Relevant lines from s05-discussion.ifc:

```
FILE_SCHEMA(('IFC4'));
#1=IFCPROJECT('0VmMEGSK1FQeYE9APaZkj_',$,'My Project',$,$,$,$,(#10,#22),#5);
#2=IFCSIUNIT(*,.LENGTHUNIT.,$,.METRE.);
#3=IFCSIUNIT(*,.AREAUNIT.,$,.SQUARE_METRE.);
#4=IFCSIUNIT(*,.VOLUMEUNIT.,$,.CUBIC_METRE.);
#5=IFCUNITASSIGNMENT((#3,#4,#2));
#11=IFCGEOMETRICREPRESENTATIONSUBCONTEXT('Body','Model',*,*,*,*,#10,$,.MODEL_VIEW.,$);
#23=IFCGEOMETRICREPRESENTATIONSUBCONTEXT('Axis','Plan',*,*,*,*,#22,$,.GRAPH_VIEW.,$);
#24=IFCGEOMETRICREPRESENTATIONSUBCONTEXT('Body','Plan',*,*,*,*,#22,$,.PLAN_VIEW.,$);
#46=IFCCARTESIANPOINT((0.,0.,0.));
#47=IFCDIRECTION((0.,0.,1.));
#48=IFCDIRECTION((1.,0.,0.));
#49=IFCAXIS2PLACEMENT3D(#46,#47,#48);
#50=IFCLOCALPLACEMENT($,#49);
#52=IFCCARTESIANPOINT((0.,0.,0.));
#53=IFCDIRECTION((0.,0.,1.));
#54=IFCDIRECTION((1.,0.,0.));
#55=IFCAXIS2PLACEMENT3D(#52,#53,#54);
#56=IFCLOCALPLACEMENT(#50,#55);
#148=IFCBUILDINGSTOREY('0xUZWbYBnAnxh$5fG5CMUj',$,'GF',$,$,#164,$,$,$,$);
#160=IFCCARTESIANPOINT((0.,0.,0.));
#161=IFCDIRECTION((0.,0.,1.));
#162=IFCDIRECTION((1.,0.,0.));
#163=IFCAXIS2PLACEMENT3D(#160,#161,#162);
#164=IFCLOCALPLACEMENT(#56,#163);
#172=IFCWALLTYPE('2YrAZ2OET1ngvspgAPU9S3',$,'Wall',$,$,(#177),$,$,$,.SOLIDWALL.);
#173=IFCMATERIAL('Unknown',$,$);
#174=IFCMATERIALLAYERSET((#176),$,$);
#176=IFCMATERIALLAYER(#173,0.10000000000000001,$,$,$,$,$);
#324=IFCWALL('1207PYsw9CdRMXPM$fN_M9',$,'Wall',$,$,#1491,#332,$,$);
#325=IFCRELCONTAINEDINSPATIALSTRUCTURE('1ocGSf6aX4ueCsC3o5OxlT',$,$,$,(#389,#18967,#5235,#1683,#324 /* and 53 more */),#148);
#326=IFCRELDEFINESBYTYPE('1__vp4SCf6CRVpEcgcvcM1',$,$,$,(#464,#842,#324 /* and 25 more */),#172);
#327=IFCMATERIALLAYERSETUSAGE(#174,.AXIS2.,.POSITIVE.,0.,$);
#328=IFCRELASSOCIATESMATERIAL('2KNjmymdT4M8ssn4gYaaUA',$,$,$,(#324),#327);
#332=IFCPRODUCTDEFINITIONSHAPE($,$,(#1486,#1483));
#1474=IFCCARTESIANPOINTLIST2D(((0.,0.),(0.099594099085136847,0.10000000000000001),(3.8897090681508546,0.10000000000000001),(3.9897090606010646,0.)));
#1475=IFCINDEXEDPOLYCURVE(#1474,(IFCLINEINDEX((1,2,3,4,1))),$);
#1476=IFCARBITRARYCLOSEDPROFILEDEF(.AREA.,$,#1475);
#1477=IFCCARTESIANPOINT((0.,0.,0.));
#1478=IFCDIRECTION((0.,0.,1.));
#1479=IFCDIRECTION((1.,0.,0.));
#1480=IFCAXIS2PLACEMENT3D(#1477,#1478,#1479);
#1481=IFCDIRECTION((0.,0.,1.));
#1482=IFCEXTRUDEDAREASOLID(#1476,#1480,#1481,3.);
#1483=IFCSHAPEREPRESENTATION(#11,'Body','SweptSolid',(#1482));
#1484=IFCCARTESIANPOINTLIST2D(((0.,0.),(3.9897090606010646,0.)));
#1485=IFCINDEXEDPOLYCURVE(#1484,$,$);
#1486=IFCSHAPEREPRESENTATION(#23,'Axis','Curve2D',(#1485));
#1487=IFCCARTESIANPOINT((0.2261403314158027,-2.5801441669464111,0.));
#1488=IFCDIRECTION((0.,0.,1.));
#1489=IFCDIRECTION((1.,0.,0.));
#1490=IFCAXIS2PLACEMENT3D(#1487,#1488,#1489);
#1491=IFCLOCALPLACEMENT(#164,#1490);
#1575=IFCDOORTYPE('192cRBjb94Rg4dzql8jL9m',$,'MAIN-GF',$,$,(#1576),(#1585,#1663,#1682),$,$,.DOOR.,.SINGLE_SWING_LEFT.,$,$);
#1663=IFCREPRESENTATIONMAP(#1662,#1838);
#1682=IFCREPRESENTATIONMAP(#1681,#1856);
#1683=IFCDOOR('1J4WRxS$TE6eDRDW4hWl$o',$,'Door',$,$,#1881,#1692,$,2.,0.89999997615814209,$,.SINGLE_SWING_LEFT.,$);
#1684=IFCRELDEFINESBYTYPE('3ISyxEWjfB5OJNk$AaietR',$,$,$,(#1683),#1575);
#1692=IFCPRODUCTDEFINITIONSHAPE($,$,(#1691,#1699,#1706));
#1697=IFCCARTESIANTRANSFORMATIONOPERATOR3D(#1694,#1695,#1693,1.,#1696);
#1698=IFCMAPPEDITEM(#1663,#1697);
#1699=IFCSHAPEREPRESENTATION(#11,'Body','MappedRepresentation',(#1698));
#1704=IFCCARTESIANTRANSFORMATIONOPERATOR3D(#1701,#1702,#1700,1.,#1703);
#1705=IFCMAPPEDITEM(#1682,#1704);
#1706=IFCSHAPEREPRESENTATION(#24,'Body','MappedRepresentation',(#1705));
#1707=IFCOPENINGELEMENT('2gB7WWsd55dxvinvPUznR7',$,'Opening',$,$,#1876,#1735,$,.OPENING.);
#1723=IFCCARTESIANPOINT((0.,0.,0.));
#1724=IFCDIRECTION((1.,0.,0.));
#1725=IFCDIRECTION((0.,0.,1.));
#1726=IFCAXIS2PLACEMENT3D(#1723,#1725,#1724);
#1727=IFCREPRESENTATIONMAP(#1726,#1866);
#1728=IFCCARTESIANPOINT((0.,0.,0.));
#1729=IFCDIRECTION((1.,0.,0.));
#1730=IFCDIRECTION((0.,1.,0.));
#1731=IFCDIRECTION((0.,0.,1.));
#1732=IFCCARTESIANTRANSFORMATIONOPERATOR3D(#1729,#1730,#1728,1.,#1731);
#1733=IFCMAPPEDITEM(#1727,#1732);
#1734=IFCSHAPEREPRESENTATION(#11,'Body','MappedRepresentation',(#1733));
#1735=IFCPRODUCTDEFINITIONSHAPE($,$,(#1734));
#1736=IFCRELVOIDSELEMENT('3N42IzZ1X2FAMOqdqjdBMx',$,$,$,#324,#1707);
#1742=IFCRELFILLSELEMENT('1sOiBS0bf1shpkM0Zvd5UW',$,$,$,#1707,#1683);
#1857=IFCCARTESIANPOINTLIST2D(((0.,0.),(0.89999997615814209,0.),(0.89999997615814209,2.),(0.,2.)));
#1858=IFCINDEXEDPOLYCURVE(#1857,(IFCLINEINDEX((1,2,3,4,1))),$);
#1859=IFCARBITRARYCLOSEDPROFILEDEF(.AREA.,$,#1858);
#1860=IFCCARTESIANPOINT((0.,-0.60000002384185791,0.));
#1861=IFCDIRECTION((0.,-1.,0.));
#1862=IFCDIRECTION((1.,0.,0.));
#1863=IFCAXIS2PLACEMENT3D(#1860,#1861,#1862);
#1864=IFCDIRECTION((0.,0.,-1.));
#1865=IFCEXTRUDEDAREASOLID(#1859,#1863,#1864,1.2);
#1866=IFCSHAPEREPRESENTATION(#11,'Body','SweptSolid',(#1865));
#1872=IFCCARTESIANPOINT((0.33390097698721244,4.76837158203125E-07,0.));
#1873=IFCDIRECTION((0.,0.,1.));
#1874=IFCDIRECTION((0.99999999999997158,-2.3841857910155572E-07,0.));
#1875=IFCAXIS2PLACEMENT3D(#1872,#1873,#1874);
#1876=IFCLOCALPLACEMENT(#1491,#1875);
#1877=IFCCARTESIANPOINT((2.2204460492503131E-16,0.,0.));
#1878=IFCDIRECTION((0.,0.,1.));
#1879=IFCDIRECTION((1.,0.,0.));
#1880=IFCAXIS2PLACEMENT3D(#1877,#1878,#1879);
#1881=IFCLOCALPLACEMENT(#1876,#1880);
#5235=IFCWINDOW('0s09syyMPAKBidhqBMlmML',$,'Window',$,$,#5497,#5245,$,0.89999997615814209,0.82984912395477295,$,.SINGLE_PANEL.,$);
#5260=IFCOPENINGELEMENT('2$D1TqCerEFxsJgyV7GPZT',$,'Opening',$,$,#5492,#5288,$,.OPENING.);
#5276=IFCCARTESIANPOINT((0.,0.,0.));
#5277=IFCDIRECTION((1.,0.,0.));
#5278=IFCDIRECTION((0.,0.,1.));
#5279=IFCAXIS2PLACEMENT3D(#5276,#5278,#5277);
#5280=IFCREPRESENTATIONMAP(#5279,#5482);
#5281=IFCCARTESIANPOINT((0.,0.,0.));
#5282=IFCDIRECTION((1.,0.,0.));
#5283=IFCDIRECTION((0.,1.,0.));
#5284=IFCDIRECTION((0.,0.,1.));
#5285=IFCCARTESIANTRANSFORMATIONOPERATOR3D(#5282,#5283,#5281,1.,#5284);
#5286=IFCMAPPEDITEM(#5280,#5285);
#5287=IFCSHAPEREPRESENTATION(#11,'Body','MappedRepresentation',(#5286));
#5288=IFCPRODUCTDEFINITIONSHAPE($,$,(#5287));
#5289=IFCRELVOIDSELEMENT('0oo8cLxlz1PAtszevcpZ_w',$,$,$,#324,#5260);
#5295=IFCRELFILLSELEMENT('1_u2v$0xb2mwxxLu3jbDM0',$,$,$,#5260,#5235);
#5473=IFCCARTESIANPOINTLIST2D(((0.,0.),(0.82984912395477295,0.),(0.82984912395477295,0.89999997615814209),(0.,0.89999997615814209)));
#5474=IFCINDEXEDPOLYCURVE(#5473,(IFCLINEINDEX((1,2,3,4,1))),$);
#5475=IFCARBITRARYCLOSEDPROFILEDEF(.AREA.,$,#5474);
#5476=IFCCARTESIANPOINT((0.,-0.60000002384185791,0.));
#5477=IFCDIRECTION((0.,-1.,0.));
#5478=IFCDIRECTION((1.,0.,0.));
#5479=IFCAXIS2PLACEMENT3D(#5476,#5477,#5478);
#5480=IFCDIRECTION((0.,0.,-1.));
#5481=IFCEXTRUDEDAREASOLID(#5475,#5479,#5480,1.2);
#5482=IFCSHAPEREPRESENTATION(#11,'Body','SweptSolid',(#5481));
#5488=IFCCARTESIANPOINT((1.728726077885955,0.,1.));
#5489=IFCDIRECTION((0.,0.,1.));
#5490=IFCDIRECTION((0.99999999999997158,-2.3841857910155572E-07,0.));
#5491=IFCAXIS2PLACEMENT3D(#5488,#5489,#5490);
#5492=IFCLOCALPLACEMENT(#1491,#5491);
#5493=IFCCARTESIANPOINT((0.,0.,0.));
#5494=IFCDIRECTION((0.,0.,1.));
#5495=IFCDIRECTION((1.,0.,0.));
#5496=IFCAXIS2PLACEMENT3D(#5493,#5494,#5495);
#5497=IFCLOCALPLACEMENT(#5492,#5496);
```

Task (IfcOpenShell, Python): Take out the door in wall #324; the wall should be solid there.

```python
import ifcopenshell
import ifcopenshell.api.feature
import ifcopenshell.api.root
import ifcopenshell.geom
import ifcopenshell.util.shape

model = ifcopenshell.open("s05-discussion.ifc")
settings = ifcopenshell.geom.settings()


def volume(element):
    """Net volume in cubic metres, openings subtracted."""
    shape = ifcopenshell.geom.create_shape(settings, element)
    return ifcopenshell.util.shape.get_volume(shape.geometry)


door = model.by_id(1683)
opening = door.FillsVoids[0].RelatingOpeningElement
wall = opening.VoidsElements[0].RelatingBuildingElement
before = volume(wall)

ifcopenshell.api.root.remove_product(model, product=door)
ifcopenshell.api.feature.remove_feature(model, feature=opening)

after = volume(wall)

print(f"wall volume {before:.3f} -> {after:.3f} m3")

model.write("s05-discussion_updated.ifc")
```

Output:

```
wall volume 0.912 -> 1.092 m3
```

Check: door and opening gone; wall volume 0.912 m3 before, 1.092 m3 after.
